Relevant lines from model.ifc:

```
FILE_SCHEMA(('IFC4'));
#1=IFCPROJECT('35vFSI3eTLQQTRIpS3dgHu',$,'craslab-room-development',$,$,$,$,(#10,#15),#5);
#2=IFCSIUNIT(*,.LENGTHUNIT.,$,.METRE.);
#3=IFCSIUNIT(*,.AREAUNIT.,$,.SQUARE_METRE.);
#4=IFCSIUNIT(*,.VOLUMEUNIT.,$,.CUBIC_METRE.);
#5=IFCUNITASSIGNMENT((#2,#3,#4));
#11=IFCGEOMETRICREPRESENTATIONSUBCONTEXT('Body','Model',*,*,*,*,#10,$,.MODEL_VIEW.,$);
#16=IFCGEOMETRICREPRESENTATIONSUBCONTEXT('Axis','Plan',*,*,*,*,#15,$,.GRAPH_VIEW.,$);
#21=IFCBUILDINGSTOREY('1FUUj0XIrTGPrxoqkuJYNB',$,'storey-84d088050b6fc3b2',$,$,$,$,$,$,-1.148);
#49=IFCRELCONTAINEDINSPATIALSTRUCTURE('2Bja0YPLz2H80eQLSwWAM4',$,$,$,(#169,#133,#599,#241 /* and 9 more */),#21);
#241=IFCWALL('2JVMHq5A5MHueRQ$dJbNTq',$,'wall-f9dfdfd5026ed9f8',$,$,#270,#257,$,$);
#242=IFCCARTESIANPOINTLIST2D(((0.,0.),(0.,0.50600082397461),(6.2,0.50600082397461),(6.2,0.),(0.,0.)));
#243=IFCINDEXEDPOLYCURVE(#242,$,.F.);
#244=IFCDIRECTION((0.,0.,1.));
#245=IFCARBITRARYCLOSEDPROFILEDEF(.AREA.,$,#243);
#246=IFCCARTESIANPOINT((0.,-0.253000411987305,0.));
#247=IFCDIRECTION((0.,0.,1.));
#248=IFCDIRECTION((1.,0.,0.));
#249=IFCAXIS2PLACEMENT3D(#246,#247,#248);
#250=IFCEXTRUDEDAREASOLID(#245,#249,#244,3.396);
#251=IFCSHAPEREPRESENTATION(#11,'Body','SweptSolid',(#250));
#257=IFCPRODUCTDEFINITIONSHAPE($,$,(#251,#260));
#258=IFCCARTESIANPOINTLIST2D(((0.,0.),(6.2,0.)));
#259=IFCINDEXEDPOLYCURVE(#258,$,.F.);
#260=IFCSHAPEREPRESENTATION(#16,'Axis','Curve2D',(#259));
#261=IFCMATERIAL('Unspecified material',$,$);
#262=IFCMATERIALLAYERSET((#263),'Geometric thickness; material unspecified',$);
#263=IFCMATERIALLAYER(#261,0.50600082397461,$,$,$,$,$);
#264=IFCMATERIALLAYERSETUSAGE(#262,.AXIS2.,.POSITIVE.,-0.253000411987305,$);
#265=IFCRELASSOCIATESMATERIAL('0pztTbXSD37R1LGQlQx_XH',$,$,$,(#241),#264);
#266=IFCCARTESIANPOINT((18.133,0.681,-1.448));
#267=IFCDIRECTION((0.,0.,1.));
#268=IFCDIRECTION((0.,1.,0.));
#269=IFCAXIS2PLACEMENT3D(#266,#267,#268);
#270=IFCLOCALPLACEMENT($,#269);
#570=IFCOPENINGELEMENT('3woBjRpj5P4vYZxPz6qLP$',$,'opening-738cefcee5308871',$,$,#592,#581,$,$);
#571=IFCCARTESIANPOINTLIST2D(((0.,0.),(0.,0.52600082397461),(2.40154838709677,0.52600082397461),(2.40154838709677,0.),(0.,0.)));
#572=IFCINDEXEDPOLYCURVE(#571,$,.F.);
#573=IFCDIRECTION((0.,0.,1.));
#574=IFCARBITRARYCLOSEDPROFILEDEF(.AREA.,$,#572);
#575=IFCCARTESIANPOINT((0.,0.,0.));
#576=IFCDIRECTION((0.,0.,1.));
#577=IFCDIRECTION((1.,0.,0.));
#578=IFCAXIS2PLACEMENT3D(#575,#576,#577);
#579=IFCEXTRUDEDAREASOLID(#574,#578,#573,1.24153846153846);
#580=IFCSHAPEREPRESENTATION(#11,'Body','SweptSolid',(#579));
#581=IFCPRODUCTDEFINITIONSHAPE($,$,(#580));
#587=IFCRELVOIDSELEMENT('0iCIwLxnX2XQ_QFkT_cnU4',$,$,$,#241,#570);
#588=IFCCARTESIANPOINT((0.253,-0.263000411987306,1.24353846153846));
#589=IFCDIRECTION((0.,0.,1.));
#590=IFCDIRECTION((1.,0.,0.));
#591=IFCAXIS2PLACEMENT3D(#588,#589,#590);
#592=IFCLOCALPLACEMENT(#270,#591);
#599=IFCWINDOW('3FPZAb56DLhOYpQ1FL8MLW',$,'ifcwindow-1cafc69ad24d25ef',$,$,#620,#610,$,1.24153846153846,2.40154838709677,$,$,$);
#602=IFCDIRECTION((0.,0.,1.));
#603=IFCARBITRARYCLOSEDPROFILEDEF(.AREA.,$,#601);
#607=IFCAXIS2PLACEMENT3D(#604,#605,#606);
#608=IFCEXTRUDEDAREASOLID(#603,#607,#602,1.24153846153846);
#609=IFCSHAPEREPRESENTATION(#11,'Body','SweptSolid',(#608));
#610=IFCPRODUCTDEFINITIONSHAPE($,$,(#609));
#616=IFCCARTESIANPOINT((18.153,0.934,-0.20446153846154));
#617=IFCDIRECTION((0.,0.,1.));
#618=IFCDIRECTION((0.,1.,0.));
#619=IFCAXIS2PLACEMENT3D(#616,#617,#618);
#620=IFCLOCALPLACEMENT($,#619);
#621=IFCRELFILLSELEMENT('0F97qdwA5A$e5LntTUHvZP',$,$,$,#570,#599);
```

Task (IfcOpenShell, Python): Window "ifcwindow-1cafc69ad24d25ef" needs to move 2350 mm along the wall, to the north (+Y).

```python
import ifcopenshell
import ifcopenshell.api.geometry
import ifcopenshell.util.placement

model = ifcopenshell.open("model.ifc")

window = model.by_guid("3FPZAb56DLhOYpQ1FL8MLW")
opening = window.FillsVoids[0].RelatingOpeningElement
wall = opening.VoidsElements[0].RelatingBuildingElement

wall_matrix = ifcopenshell.util.placement.get_local_placement(wall.ObjectPlacement)
shift = wall_matrix[:3, 0] * 2.35
before = ifcopenshell.util.placement.get_local_placement(window.ObjectPlacement)[:3, 3].copy()

# The window is not placed relative to its opening, so move both.
for product in (opening, window):
    matrix = ifcopenshell.util.placement.get_local_placement(product.ObjectPlacement)
    matrix[:3, 3] += shift
    ifcopenshell.api.geometry.edit_object_placement(model, product=product, matrix=matrix, is_si=False)

after = ifcopenshell.util.placement.get_local_placement(window.ObjectPlacement)[:3, 3]
print("window moved by", (after - before).round(3) + 0.0)

model.write("model-out.ifc")
```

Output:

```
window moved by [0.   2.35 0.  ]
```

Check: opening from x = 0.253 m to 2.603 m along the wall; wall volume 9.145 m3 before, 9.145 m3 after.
